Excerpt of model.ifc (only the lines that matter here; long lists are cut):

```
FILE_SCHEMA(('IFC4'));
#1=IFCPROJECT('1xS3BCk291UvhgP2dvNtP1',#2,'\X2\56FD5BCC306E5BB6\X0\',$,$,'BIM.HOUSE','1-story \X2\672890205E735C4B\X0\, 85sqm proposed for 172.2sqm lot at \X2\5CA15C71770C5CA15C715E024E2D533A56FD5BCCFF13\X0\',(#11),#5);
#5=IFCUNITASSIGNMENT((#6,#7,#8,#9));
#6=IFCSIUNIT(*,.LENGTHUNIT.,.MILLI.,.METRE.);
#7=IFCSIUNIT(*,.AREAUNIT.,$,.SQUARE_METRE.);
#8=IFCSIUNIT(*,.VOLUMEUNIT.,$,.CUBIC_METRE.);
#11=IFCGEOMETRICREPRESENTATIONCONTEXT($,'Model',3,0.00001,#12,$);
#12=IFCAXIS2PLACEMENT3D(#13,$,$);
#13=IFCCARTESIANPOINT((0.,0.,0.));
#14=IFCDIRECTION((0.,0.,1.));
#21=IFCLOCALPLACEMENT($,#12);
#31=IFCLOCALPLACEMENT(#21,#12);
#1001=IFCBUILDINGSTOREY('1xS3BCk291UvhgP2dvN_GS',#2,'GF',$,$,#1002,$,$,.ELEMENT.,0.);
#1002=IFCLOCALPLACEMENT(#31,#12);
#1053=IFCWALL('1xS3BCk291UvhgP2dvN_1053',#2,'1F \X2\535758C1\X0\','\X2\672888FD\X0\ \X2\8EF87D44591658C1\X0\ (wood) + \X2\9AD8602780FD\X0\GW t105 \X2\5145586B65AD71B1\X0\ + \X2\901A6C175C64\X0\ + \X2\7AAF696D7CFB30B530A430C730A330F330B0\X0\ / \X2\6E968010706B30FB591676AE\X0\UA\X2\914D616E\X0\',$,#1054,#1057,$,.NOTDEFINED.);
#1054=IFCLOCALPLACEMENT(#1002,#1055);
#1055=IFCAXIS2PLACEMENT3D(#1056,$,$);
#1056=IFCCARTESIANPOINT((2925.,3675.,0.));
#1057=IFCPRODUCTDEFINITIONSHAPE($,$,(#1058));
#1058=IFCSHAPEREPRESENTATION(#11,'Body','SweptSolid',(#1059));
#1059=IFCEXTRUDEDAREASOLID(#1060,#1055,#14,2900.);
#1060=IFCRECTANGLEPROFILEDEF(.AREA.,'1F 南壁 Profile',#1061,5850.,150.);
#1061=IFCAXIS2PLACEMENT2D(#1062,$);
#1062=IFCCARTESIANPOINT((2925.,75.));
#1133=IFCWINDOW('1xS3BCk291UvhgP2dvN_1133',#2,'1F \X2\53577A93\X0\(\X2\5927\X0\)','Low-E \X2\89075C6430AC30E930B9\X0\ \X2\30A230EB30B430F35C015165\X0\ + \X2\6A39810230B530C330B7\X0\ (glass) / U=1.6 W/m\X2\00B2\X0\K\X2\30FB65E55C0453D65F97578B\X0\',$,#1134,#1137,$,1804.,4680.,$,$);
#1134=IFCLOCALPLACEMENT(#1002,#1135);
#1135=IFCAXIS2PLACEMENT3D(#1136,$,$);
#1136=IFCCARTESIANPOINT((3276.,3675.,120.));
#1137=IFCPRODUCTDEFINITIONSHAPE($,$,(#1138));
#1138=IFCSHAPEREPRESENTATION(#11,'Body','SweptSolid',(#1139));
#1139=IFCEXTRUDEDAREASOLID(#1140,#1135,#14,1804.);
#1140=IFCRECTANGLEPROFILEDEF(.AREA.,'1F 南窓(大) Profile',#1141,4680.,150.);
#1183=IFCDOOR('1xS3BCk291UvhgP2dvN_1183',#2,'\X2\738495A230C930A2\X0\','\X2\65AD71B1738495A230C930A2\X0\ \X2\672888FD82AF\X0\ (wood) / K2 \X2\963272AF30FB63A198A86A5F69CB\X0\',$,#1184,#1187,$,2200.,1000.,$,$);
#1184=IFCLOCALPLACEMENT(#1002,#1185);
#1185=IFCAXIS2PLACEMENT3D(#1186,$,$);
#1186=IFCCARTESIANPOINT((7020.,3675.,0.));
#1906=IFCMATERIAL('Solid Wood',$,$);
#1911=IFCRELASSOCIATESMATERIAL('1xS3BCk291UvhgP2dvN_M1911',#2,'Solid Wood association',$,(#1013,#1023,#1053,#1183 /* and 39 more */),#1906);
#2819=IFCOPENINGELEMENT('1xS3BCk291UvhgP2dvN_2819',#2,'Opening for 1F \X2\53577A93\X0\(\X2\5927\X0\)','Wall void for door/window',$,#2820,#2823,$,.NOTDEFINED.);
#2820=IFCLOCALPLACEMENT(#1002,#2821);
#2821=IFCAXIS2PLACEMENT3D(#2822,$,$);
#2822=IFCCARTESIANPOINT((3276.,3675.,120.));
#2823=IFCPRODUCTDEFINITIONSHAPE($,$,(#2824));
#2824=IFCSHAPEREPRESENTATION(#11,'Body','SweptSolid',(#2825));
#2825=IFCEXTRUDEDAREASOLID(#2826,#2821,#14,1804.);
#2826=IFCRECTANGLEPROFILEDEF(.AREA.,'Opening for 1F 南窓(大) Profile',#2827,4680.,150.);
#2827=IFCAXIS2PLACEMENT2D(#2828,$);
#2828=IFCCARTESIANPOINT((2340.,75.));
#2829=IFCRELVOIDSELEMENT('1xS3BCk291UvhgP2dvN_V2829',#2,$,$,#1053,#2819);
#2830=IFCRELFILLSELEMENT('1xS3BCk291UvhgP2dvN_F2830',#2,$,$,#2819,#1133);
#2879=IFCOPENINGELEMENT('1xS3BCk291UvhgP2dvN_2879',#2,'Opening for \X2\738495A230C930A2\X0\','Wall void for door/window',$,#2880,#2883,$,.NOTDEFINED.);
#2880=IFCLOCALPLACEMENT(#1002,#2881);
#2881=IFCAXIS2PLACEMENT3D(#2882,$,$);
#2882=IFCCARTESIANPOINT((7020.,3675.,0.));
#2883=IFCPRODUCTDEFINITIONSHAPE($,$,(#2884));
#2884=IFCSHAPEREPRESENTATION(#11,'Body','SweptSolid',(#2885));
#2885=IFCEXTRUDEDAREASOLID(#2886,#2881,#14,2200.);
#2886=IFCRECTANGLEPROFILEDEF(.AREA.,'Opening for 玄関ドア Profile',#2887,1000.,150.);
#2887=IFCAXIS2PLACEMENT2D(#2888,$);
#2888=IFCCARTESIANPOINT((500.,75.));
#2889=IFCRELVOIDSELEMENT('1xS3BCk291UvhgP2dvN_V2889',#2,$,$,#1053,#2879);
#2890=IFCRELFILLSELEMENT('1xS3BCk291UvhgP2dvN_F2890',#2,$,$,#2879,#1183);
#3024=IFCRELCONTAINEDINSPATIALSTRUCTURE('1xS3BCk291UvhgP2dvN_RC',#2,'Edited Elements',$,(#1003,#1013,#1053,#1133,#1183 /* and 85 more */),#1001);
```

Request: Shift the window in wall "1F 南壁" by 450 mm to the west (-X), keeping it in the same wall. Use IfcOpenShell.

```python
import ifcopenshell
import ifcopenshell.api.geometry
import ifcopenshell.util.placement

model = ifcopenshell.open("model.ifc")

window = model.by_id(1133)
opening = window.FillsVoids[0].RelatingOpeningElement
wall = opening.VoidsElements[0].RelatingBuildingElement

wall_matrix = ifcopenshell.util.placement.get_local_placement(wall.ObjectPlacement)
shift = wall_matrix[:3, 0] * -450.0
before = ifcopenshell.util.placement.get_local_placement(window.ObjectPlacement)[:3, 3].copy()

# The window is not placed relative to its opening, so move both.
for product in (opening, window):
    matrix = ifcopenshell.util.placement.get_local_placement(product.ObjectPlacement)
    matrix[:3, 3] += shift
    ifcopenshell.api.geometry.edit_object_placement(model, product=product, matrix=matrix, is_si=False)

after = ifcopenshell.util.placement.get_local_placement(window.ObjectPlacement)[:3, 3]
print("window moved by", (after - before).round(3) + 0.0)

model.write("model_updated.ifc")
```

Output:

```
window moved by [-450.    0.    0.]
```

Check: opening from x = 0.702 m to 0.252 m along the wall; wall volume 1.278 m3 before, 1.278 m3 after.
